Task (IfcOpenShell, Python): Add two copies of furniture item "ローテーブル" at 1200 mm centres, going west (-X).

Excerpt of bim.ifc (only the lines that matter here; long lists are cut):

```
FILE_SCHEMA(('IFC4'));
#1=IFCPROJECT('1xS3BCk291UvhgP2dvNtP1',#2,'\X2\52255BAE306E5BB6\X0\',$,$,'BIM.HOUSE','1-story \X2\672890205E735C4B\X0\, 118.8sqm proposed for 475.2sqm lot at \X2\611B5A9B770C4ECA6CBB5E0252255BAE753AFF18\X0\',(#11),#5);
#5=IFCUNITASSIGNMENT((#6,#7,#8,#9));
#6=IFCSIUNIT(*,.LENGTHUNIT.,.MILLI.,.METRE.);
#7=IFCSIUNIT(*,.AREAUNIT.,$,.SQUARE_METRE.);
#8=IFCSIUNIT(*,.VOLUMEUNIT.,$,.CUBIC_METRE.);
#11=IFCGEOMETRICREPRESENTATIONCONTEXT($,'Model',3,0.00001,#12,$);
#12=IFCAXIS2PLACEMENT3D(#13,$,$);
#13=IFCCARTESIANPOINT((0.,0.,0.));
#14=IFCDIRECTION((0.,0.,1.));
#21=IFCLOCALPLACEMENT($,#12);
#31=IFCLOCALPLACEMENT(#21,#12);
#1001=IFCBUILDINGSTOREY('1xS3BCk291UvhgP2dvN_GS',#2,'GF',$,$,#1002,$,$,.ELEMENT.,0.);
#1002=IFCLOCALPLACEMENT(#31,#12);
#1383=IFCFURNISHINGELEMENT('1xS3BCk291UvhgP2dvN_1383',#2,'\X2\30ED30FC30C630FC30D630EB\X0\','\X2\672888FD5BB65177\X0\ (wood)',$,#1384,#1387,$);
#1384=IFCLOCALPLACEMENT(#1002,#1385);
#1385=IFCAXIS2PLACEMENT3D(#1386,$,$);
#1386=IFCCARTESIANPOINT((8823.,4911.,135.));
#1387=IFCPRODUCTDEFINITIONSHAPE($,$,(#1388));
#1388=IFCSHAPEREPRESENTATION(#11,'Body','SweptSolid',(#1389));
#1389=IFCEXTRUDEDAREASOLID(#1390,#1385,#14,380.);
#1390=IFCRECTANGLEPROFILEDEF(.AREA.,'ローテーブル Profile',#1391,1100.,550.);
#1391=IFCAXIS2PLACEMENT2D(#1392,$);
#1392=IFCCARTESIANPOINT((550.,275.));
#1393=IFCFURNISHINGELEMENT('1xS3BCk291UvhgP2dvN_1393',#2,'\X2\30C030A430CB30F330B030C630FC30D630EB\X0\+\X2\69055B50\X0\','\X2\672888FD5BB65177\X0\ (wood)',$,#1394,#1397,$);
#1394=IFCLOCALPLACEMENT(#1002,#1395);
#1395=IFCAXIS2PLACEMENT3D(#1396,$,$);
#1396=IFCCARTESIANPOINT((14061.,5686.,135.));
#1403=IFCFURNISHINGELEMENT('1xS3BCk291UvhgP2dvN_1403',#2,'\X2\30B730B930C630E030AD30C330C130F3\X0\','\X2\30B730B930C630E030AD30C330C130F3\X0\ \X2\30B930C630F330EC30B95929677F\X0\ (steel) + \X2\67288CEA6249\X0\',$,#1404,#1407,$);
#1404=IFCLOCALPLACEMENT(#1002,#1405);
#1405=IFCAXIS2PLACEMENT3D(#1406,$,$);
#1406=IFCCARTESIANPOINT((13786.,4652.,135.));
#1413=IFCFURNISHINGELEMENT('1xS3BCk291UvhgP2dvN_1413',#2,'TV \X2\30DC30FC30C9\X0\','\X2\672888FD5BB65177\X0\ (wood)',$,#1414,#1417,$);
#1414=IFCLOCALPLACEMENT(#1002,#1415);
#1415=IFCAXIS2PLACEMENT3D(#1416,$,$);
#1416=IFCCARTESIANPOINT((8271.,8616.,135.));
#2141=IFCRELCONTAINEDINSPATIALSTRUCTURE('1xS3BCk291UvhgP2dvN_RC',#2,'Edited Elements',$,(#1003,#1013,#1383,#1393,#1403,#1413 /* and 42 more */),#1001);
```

```python
import numpy as np
import ifcopenshell
import ifcopenshell.api.geometry
import ifcopenshell.api.root
import ifcopenshell.util.element
import ifcopenshell.util.placement
import ifcopenshell.util.unit

model = ifcopenshell.open("bim.ifc")
unit_scale = ifcopenshell.util.unit.calculate_unit_scale(model)


def reuse_history(source, copy):
    """copy_class also copies each property set's owner history, people and application; keep the originals."""
    for rel in copy.IsDefinedBy:
        if rel.is_a("IfcRelDefinesByProperties") and (history := rel.RelatingPropertyDefinition.OwnerHistory):
            rel.RelatingPropertyDefinition.OwnerHistory = source.OwnerHistory
            ifcopenshell.util.element.remove_deep2(model, history)


source = model.by_guid("1xS3BCk291UvhgP2dvN_1383")
base = ifcopenshell.util.placement.get_local_placement(source.ObjectPlacement)
step = np.array([-1.0, 0.0, 0.0]) * 1.2 / unit_scale

for i in range(1, 3):
    copy = ifcopenshell.api.root.copy_class(model, product=source)
    copy.Representation = ifcopenshell.util.element.copy_deep(
        model, source.Representation, exclude=["IfcGeometricRepresentationContext", "IfcRepresentationMap"]
    )
    reuse_history(source, copy)
    matrix = base.copy()
    matrix[:3, 3] += i * step
    print("added at", matrix[:3, 3].round(3) + 0.0)
    ifcopenshell.api.geometry.edit_object_placement(model, product=copy, matrix=matrix, is_si=False)

model.write("bim_rev.ifc")
```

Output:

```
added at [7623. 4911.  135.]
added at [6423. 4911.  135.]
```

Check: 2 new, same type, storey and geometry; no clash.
